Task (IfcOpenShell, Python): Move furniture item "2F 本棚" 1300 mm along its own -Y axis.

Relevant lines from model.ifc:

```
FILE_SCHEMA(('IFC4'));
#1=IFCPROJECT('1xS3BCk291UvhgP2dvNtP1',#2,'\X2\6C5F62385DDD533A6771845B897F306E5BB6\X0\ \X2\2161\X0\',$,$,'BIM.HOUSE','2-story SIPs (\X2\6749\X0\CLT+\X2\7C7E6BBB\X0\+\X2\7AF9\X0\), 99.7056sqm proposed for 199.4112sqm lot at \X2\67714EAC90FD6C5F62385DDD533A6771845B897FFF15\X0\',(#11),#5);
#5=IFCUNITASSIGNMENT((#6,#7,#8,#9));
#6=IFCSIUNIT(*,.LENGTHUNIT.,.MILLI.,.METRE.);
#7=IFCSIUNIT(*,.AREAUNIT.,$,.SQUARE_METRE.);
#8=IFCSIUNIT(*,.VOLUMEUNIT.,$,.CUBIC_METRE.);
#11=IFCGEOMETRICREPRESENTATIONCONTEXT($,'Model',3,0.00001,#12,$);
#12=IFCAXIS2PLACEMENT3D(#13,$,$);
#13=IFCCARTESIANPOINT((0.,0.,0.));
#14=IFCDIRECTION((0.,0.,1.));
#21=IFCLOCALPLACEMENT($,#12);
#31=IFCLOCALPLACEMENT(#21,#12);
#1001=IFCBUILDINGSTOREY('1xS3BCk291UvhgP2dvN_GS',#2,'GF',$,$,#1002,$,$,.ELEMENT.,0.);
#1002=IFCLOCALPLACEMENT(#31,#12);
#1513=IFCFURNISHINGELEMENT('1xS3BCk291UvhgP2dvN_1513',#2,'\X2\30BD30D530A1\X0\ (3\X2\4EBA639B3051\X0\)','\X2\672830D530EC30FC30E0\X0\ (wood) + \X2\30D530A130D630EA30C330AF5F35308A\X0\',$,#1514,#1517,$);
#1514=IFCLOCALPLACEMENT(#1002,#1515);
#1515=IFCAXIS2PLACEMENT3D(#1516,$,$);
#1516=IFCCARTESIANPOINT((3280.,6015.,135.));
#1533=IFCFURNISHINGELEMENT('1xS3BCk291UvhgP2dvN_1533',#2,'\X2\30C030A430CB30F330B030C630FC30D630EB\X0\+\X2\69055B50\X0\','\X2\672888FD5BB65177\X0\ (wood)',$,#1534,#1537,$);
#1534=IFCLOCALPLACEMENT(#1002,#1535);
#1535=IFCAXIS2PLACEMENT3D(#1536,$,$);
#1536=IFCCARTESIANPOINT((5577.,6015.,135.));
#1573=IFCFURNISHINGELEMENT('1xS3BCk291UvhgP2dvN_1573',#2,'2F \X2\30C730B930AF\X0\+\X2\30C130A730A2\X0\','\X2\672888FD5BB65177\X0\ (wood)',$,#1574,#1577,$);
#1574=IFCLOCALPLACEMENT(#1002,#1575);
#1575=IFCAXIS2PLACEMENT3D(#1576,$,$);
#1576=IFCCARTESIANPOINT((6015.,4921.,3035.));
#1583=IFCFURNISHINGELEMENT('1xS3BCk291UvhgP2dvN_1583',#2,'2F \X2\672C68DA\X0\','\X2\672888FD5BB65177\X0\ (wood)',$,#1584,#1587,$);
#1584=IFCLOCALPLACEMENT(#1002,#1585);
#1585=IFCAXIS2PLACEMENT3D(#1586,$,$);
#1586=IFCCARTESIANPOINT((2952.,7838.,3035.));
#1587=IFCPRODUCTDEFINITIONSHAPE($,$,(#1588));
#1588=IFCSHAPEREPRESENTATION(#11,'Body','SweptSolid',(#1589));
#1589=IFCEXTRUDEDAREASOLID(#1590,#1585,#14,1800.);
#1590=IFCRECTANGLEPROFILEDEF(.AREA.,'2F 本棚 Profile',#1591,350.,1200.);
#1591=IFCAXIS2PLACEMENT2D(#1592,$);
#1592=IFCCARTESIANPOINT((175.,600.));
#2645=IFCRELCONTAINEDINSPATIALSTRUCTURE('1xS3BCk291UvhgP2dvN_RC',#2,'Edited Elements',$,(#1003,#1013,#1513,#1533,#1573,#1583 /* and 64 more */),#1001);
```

```python
import ifcopenshell
import ifcopenshell.api.geometry
import ifcopenshell.util.placement

model = ifcopenshell.open("model.ifc")

item = model.by_guid("1xS3BCk291UvhgP2dvN_1583")
matrix = ifcopenshell.util.placement.get_local_placement(item.ObjectPlacement)
matrix[:3, 3] -= matrix[:3, 1] * 1300.0
ifcopenshell.api.geometry.edit_object_placement(model, product=item, matrix=matrix, is_si=False)

print(ifcopenshell.util.placement.get_local_placement(item.ObjectPlacement).round(3) + 0.0)

model.write("model_edited.ifc")
```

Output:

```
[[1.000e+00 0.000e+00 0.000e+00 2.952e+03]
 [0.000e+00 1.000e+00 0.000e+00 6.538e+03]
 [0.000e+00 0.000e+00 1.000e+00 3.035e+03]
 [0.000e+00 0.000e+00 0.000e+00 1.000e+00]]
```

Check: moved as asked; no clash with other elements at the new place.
